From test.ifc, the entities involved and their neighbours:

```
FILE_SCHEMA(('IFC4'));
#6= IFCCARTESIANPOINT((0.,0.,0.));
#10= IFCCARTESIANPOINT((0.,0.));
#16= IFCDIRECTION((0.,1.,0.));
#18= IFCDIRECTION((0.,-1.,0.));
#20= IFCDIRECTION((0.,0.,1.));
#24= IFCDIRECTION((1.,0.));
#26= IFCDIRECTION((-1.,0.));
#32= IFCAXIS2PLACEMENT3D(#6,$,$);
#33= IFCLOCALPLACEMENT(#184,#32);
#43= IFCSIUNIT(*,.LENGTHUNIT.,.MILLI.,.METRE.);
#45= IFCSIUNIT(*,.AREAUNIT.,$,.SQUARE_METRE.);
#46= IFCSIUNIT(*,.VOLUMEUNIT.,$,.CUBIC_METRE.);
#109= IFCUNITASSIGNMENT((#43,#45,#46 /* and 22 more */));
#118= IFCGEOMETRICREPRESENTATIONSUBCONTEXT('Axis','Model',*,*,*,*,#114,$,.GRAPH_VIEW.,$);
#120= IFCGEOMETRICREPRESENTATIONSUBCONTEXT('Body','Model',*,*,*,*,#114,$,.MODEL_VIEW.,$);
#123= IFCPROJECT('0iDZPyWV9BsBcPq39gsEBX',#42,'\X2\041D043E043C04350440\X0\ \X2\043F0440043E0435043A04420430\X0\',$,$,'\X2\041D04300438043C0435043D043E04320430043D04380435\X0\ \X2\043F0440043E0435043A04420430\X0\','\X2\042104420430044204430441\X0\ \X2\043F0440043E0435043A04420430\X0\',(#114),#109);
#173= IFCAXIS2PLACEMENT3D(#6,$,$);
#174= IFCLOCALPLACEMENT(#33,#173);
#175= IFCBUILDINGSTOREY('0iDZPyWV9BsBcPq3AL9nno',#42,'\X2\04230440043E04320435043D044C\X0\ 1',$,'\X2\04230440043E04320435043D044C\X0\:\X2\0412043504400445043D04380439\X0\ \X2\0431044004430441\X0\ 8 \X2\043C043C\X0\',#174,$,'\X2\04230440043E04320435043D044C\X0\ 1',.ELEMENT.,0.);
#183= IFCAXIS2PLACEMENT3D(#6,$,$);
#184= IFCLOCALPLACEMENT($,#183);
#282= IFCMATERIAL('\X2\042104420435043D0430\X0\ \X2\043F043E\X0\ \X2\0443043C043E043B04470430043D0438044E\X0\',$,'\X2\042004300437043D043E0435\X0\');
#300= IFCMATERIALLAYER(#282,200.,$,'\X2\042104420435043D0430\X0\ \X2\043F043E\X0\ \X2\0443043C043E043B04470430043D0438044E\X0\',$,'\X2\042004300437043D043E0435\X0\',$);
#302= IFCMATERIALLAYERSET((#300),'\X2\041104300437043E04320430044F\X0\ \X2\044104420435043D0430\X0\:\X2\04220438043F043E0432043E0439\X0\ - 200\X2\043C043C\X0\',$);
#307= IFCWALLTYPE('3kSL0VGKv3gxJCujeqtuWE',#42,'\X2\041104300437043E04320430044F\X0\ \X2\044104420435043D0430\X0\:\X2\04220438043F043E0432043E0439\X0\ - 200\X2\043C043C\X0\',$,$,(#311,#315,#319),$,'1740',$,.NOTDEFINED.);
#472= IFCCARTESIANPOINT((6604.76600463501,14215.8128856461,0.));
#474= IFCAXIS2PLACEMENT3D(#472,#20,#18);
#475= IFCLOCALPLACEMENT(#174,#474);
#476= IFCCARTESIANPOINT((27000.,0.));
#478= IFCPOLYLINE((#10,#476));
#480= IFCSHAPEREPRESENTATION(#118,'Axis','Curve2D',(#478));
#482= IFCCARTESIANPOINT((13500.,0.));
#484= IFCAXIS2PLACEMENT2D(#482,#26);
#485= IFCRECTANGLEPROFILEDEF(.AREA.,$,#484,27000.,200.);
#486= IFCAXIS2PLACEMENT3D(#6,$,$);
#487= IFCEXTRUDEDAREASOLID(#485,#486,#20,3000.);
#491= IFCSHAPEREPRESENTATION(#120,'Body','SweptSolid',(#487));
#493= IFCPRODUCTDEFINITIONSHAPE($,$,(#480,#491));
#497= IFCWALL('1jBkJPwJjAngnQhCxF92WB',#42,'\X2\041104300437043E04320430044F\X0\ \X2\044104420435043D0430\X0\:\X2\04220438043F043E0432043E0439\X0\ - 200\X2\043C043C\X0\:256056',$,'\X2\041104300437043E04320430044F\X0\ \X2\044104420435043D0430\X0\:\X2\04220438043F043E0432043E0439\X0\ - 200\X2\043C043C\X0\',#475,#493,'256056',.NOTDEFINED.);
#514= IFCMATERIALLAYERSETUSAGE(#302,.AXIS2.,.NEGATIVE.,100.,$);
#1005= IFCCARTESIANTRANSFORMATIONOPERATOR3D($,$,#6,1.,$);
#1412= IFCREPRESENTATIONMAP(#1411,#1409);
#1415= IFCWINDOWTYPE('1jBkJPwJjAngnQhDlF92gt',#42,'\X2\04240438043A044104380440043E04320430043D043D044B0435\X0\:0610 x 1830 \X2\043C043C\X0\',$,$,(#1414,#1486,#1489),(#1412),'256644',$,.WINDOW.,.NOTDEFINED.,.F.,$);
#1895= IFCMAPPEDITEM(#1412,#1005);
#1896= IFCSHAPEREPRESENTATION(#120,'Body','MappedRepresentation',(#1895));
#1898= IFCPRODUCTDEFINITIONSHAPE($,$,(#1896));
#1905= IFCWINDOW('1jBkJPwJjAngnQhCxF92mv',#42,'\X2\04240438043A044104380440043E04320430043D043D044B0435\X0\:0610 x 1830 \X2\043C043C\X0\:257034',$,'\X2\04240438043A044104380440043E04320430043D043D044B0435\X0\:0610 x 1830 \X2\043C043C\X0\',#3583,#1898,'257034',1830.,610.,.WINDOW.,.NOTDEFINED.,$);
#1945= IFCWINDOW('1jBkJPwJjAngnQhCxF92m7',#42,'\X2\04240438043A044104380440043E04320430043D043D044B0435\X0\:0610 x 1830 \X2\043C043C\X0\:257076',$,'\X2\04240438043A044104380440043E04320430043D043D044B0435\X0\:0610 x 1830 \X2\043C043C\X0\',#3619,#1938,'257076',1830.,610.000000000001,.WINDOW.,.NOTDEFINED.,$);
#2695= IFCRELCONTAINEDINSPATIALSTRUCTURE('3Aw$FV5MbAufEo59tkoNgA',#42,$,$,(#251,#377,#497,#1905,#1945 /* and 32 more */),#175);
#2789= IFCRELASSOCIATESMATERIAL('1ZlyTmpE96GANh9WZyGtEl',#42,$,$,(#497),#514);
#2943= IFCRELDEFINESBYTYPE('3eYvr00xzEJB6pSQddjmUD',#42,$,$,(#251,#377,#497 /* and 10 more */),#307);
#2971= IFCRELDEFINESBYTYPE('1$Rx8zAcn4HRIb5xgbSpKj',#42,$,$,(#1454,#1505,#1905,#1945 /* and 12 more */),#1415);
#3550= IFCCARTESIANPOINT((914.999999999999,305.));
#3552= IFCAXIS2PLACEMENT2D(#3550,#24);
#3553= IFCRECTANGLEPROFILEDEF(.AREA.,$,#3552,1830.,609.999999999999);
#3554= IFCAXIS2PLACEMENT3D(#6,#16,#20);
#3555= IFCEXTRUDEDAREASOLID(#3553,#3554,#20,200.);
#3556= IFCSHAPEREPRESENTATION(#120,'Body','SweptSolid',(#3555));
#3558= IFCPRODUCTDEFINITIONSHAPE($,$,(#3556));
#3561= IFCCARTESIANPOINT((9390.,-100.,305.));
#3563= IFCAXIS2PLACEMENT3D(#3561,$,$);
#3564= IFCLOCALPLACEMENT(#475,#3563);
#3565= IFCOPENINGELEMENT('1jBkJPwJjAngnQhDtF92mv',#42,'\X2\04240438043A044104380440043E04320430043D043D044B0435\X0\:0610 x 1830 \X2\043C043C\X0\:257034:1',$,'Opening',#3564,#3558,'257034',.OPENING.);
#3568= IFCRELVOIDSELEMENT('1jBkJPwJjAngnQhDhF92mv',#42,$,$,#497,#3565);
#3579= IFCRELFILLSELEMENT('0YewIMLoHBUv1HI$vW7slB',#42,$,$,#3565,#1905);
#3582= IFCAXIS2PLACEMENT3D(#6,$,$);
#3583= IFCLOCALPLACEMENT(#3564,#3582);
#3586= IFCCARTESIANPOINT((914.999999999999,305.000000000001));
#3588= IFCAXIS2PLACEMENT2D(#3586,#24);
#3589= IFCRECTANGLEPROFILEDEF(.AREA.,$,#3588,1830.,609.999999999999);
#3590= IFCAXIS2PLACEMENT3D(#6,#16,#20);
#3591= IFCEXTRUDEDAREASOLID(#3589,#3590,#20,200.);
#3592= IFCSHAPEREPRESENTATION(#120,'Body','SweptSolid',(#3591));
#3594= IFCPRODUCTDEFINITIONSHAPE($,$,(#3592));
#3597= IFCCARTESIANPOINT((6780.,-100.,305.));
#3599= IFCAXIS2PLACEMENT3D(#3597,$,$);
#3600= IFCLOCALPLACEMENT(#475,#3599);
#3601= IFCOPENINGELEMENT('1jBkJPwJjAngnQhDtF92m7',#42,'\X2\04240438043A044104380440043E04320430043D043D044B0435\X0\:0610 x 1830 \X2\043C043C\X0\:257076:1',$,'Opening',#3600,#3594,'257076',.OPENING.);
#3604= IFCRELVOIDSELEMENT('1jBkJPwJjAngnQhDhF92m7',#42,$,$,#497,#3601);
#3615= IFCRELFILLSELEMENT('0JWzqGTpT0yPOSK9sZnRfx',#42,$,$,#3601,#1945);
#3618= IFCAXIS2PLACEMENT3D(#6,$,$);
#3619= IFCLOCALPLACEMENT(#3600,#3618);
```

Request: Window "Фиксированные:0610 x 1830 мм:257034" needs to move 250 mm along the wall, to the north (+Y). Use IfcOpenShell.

```python
import ifcopenshell
import ifcopenshell.api.geometry
import ifcopenshell.util.placement
import ifcopenshell.util.unit

model = ifcopenshell.open("test.ifc")
unit_scale = ifcopenshell.util.unit.calculate_unit_scale(model)

window = model.by_guid("1jBkJPwJjAngnQhCxF92mv")
opening = window.FillsVoids[0].RelatingOpeningElement
wall = opening.VoidsElements[0].RelatingBuildingElement

wall_matrix = ifcopenshell.util.placement.get_local_placement(wall.ObjectPlacement)
shift = wall_matrix[:3, 0] * -0.25 / unit_scale
before = ifcopenshell.util.placement.get_local_placement(window.ObjectPlacement)[:3, 3].copy()

# The window is placed relative to its opening, so it follows when the opening moves.
matrix = ifcopenshell.util.placement.get_local_placement(opening.ObjectPlacement)
matrix[:3, 3] += shift
ifcopenshell.api.geometry.edit_object_placement(
    model, product=opening, matrix=matrix, is_si=False, should_transform_children=True
)

after = ifcopenshell.util.placement.get_local_placement(window.ObjectPlacement)[:3, 3]
print("window moved by", (after - before).round(3) + 0.0)

model.write("test_rev.ifc")
```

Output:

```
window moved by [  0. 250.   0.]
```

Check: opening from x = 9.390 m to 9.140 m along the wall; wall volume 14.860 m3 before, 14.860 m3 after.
